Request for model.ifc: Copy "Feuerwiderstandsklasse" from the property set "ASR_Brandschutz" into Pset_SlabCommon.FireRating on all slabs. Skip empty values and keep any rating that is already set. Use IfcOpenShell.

First a look at what the model holds.

```python
import ifcopenshell
import ifcopenshell.util.element

model = ifcopenshell.open("model.ifc")
print(model.schema)
slabs = model.by_type("IfcSlab")
print(len(slabs), "slabs")
for e in slabs[:8]:
    source = ifcopenshell.util.element.get_pset(e, "ASR_Brandschutz", "Feuerwiderstandsklasse")
    target = ifcopenshell.util.element.get_pset(e, "Pset_SlabCommon", "FireRating")
    print(e.id(), repr(source), repr(target), sep=" | ")
```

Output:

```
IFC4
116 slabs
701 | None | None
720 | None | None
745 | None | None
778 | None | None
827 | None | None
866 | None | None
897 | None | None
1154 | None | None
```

```python
import ifcopenshell
import ifcopenshell.api.pset
import ifcopenshell.util.element

model = ifcopenshell.open("model.ifc")

count = 0
for e in model.by_type("IfcSlab"):
    value = ifcopenshell.util.element.get_pset(e, "ASR_Brandschutz", "Feuerwiderstandsklasse")
    current = ifcopenshell.util.element.get_pset(e, "Pset_SlabCommon", "FireRating")
    if not value or not value.strip() or current:
        continue
    # add_pset returns the element's existing set when there is one.
    pset = ifcopenshell.api.pset.add_pset(model, product=e, name="Pset_SlabCommon")
    ifcopenshell.api.pset.edit_pset(model, pset=pset, properties={"FireRating": value})
    count += 1

print(count, "slabs updated")

model.write("model-out.ifc")
```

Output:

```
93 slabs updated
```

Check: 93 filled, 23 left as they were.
